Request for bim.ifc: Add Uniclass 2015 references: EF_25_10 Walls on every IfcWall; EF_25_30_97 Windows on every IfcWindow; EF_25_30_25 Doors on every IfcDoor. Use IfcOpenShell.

First a look at what the model holds.

```python
import ifcopenshell

model = ifcopenshell.open("bim.ifc")
print(model.schema)
print("classifications:", [c.Name for c in model.by_type("IfcClassification")])
for ifc_class in ("IfcDoor", "IfcRoof", "IfcStair", "IfcWall", "IfcWindow"):
    print(ifc_class, len(model.by_type(ifc_class)))
```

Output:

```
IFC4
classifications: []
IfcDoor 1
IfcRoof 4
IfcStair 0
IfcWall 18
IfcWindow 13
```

```python
import ifcopenshell
import ifcopenshell.api.classification

model = ifcopenshell.open("bim.ifc")

system = ifcopenshell.api.classification.add_classification(model, classification="Uniclass 2015")

codes = {
    "IfcWall": ("EF_25_10", "Walls"),
    "IfcWindow": ("EF_25_30_97", "Windows"),
    "IfcDoor": ("EF_25_30_25", "Doors"),
}
for ifc_class, (code, name) in codes.items():
    products = model.by_type(ifc_class)
    ifcopenshell.api.classification.add_reference(
        model, products=products, classification=system, identification=code, name=name
    )
    print(code, len(products))

model.write("bim_updated.ifc")
```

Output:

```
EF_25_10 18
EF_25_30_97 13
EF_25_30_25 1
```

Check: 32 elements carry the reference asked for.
